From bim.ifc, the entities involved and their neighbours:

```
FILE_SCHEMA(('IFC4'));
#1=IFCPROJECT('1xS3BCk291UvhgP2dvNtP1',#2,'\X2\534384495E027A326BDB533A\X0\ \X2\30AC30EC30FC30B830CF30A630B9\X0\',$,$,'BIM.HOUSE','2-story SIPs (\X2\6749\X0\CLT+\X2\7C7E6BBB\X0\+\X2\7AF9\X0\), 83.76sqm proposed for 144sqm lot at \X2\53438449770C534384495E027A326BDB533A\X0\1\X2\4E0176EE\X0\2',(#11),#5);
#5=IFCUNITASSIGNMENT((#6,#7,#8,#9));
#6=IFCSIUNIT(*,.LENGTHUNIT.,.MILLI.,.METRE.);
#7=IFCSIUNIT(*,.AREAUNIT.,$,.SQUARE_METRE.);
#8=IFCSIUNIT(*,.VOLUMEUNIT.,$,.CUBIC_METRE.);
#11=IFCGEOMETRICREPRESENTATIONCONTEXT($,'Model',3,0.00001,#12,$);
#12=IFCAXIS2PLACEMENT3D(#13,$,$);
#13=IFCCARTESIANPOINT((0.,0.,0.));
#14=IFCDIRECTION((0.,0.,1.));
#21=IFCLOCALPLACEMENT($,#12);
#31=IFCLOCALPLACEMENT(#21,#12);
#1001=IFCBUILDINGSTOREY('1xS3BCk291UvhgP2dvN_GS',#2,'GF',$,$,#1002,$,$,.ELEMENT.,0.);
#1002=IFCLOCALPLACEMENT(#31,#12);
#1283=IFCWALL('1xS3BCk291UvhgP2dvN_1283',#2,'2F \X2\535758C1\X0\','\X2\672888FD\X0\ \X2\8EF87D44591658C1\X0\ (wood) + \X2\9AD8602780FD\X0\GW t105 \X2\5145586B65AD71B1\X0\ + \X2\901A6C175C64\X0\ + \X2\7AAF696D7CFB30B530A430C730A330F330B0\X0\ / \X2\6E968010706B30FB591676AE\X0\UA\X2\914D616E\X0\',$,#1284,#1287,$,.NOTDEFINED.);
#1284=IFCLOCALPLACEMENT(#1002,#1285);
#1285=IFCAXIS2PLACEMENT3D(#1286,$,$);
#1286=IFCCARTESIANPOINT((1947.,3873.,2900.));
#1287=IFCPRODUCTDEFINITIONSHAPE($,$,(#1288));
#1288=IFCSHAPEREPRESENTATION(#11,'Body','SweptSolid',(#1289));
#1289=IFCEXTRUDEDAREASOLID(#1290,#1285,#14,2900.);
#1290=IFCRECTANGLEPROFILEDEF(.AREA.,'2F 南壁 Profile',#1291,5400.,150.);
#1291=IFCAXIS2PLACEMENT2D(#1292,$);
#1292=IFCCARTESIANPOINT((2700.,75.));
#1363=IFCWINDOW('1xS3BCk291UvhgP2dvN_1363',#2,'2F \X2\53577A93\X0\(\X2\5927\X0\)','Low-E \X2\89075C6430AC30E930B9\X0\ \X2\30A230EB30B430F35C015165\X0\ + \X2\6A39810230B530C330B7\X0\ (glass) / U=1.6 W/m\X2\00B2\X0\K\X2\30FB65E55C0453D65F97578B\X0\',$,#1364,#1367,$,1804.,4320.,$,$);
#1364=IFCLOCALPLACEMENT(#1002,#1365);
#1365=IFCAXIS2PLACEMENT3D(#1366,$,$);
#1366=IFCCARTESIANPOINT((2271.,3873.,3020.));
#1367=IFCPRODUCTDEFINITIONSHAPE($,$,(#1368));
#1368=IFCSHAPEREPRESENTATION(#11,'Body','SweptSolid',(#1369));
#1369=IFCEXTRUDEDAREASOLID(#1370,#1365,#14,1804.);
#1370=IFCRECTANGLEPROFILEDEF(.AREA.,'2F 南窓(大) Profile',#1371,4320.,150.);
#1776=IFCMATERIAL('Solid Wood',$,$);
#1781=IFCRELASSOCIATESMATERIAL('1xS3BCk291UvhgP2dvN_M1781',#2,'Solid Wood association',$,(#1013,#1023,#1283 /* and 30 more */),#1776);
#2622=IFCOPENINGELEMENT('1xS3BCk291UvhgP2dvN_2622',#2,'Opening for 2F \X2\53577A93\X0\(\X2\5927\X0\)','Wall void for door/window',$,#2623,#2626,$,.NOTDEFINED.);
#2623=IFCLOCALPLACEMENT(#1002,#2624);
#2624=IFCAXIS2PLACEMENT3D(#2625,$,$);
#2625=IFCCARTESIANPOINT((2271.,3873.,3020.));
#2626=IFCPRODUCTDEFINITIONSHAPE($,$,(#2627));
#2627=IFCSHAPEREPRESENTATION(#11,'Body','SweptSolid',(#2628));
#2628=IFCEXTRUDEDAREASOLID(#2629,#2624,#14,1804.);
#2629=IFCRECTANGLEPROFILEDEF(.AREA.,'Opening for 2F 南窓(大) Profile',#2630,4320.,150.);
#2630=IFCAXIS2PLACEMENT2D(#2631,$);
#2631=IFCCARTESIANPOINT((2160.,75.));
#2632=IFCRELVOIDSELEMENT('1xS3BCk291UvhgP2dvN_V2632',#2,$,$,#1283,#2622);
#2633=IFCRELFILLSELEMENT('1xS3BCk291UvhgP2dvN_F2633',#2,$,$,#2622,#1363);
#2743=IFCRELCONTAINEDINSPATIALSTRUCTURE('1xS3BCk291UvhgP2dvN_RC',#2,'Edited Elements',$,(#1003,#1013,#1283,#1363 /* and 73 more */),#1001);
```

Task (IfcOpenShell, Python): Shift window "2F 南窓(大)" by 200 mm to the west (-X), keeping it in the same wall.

```python
import ifcopenshell
import ifcopenshell.api.geometry
import ifcopenshell.util.placement

model = ifcopenshell.open("bim.ifc")

window = model.by_guid("1xS3BCk291UvhgP2dvN_1363")
opening = window.FillsVoids[0].RelatingOpeningElement
wall = opening.VoidsElements[0].RelatingBuildingElement

wall_matrix = ifcopenshell.util.placement.get_local_placement(wall.ObjectPlacement)
shift = wall_matrix[:3, 0] * -200.0
before = ifcopenshell.util.placement.get_local_placement(window.ObjectPlacement)[:3, 3].copy()

# The window is not placed relative to its opening, so move both.
for product in (opening, window):
    matrix = ifcopenshell.util.placement.get_local_placement(product.ObjectPlacement)
    matrix[:3, 3] += shift
    ifcopenshell.api.geometry.edit_object_placement(model, product=product, matrix=matrix, is_si=False)

after = ifcopenshell.util.placement.get_local_placement(window.ObjectPlacement)[:3, 3]
print("window moved by", (after - before).round(3) + 0.0)

model.write("bim_updated.ifc")
```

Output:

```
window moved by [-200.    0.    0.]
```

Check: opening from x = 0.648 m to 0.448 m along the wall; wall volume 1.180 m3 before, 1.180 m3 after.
